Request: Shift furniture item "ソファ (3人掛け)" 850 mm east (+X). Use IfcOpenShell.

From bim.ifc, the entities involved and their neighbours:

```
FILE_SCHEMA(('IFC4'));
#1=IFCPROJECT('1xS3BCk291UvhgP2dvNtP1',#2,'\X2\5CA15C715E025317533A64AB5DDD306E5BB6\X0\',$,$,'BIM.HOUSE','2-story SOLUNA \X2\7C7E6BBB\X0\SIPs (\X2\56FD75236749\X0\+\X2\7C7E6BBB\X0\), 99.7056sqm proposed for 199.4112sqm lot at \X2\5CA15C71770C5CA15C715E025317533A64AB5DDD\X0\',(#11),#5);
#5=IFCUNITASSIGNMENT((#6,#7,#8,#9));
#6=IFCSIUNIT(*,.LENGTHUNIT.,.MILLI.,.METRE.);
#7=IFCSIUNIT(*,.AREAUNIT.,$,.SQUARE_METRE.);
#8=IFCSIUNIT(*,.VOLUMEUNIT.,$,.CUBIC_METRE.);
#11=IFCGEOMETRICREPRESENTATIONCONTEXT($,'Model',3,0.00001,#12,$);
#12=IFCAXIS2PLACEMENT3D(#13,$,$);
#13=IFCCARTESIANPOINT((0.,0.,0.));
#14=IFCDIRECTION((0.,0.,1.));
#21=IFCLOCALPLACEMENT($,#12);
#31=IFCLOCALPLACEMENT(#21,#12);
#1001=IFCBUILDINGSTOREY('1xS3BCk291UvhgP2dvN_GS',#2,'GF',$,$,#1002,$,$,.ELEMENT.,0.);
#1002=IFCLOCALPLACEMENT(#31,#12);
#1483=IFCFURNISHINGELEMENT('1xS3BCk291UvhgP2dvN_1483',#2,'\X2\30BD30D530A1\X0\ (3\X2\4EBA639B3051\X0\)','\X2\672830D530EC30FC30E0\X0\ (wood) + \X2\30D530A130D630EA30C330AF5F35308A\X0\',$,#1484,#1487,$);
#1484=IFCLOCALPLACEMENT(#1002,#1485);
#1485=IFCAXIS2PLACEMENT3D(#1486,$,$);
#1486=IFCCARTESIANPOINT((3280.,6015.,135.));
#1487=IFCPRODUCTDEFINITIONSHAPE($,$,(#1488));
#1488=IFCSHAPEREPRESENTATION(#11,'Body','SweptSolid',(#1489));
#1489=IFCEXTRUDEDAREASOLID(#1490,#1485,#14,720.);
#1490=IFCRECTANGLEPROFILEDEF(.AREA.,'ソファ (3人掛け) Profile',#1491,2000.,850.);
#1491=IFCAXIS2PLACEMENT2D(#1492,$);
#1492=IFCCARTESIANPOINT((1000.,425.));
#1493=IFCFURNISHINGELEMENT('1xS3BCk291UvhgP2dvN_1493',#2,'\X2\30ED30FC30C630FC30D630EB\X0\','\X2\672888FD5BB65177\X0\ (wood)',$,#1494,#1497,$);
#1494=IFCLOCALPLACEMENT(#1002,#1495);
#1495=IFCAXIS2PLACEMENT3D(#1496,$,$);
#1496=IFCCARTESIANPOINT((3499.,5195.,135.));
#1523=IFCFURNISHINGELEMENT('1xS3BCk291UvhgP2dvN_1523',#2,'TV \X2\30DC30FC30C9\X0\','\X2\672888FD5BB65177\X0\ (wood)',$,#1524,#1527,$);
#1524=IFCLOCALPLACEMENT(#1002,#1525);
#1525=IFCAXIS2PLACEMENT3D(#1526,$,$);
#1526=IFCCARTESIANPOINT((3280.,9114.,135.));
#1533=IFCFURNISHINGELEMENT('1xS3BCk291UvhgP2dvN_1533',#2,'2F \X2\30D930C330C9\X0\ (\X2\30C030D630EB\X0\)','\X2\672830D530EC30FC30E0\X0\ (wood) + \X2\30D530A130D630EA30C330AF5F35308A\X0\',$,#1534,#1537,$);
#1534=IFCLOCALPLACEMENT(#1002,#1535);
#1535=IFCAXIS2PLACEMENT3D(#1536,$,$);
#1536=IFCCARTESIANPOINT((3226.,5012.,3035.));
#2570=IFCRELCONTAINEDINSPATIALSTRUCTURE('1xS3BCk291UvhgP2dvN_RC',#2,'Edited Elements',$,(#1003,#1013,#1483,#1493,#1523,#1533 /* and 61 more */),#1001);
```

```python
import ifcopenshell
import ifcopenshell.api.geometry
import ifcopenshell.util.placement
import ifcopenshell.util.unit

model = ifcopenshell.open("bim.ifc")
unit_scale = ifcopenshell.util.unit.calculate_unit_scale(model)

item = model.by_guid("1xS3BCk291UvhgP2dvN_1483")
matrix = ifcopenshell.util.placement.get_local_placement(item.ObjectPlacement)
matrix[0, 3] += 0.85 / unit_scale
ifcopenshell.api.geometry.edit_object_placement(model, product=item, matrix=matrix, is_si=False)

print(ifcopenshell.util.placement.get_local_placement(item.ObjectPlacement).round(3) + 0.0)

model.write("bim_edited.ifc")
```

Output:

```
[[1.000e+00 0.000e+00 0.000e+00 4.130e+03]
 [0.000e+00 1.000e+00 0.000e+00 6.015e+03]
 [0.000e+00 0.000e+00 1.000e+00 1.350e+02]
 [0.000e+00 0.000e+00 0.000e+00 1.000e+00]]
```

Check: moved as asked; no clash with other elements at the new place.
